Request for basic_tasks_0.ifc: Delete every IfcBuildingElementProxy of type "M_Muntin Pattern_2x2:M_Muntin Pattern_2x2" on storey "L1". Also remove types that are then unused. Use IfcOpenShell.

First a look at what the model holds.

```python
import ifcopenshell
import ifcopenshell.util.element

model = ifcopenshell.open("basic_tasks_0.ifc")
print(model.schema)
storey = next(s for s in model.by_type("IfcBuildingStorey") if s.Name == "L1")
proxies = [e for e in ifcopenshell.util.element.get_decomposition(storey) if e.is_a("IfcBuildingElementProxy")]
seen = {}
for e in proxies:
    element_type = ifcopenshell.util.element.get_type(e)
    name = element_type.Name if element_type not in (None, e) else None
    seen[name] = seen.get(name, 0) + 1
for name, count in sorted(seen.items(), key=str):
    print(count, "x", name)
```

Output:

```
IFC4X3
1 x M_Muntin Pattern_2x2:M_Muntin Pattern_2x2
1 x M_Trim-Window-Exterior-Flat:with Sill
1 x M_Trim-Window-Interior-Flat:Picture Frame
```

```python
import ifcopenshell
import ifcopenshell.api.root
import ifcopenshell.util.element

model = ifcopenshell.open("basic_tasks_0.ifc")

storey = next(s for s in model.by_type("IfcBuildingStorey") if s.Name == "L1")
proxies = [e for e in ifcopenshell.util.element.get_decomposition(storey) if e.is_a("IfcBuildingElementProxy")]
targets = [e for e in proxies if (t := ifcopenshell.util.element.get_type(e)) not in (None, e) and t.Name == "M_Muntin Pattern_2x2:M_Muntin Pattern_2x2"]
types = {ifcopenshell.util.element.get_type(e) for e in targets} - {None, *targets}

for e in targets:
    ifcopenshell.api.root.remove_product(model, product=e)
print(len(targets), "removed")

unused = [t for t in types if not ifcopenshell.util.element.get_types(t)]
for t in unused:
    ifcopenshell.api.root.remove_product(model, product=t)
print(len(unused), "unused types removed")

model.write("basic_tasks_0_updated.ifc")
```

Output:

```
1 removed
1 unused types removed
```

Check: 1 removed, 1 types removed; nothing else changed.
